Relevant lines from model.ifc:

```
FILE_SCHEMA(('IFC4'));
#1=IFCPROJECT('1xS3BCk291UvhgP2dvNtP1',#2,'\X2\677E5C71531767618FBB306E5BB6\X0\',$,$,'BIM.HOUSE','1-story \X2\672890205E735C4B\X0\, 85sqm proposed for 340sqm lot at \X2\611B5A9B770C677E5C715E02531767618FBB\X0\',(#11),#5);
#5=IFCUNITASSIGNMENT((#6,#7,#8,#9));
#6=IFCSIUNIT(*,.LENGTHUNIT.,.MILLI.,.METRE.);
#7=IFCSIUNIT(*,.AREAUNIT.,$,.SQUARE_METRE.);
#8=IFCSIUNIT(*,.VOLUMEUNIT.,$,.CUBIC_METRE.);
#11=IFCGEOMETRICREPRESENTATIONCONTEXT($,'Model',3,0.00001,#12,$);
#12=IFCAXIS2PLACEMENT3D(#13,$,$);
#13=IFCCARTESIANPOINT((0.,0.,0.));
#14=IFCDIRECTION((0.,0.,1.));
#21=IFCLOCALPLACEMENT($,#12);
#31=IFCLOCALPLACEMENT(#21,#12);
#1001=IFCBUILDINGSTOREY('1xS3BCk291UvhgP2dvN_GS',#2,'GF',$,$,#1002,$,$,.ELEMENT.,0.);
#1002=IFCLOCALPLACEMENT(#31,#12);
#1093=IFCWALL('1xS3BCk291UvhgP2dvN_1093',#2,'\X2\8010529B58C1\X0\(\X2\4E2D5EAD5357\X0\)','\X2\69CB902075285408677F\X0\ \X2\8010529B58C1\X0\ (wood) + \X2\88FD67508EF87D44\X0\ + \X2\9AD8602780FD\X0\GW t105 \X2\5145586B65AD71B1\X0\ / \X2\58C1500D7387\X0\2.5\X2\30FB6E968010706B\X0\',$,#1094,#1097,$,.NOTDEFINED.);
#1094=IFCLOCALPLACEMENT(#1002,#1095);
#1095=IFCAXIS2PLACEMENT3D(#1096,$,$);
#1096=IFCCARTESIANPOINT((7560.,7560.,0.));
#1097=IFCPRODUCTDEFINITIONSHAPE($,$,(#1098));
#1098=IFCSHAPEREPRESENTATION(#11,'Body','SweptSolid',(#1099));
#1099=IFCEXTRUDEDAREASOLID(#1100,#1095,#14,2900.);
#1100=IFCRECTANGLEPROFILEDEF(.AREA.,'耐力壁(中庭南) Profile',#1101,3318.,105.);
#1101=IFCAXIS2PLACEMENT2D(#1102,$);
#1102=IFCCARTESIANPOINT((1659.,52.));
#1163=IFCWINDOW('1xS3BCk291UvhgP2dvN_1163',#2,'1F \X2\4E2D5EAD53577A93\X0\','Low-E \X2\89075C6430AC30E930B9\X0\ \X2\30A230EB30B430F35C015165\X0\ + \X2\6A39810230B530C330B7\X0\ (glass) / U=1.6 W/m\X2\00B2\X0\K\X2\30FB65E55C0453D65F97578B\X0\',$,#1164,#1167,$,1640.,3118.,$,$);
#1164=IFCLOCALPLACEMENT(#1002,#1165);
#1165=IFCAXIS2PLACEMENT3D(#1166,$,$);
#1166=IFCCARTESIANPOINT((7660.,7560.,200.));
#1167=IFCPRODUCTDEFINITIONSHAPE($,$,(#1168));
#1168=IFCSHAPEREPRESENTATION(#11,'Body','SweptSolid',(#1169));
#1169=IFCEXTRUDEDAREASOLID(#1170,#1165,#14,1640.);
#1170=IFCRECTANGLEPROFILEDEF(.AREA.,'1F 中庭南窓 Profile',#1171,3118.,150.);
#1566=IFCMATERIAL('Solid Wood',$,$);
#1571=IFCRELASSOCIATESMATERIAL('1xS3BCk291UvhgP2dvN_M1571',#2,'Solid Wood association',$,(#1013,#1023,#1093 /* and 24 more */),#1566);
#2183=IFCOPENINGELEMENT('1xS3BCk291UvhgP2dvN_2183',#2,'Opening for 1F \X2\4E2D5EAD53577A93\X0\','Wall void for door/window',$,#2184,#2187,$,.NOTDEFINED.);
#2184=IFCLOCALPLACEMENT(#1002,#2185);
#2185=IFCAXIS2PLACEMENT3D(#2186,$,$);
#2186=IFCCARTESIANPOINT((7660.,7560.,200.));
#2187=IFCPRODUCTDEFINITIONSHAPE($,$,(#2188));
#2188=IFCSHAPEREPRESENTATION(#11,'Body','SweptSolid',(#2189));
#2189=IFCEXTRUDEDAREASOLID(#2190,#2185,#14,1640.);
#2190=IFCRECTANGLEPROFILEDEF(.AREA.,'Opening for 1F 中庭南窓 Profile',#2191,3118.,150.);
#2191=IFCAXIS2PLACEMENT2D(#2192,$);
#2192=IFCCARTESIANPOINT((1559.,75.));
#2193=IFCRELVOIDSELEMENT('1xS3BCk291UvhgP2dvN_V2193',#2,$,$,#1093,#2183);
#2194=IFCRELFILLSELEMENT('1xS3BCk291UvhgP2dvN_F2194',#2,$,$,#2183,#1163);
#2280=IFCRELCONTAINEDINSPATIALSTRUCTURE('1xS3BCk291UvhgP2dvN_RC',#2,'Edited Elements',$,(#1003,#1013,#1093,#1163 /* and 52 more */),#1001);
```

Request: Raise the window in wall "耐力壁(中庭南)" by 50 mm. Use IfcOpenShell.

```python
import numpy as np
import ifcopenshell
import ifcopenshell.api.geometry
import ifcopenshell.util.placement
import ifcopenshell.util.unit

model = ifcopenshell.open("model.ifc")
unit_scale = ifcopenshell.util.unit.calculate_unit_scale(model)

window = model.by_id(1163)
opening = window.FillsVoids[0].RelatingOpeningElement
dz = 0.05 / unit_scale

shift = np.array([0.0, 0.0, dz])
# The window is not placed relative to its opening, so move both.
for product in (opening, window):
    matrix = ifcopenshell.util.placement.get_local_placement(product.ObjectPlacement)
    matrix[:3, 3] += shift
    ifcopenshell.api.geometry.edit_object_placement(model, product=product, matrix=matrix, is_si=False)

print(f"moved by {dz * unit_scale:+.3f} m")

model.write("model-out.ifc")
```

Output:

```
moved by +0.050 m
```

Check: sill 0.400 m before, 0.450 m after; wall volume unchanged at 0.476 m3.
